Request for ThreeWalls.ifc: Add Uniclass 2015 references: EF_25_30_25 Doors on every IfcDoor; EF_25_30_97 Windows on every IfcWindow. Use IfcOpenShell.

First a look at what the model holds.

```python
import ifcopenshell

model = ifcopenshell.open("ThreeWalls.ifc")
print(model.schema)
print("classifications:", [c.Name for c in model.by_type("IfcClassification")])
for ifc_class in ("IfcDoor", "IfcRoof", "IfcStair", "IfcWall", "IfcWindow"):
    print(ifc_class, len(model.by_type(ifc_class)))
```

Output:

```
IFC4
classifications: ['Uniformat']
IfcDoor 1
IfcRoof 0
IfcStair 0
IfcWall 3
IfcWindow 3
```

```python
import ifcopenshell
import ifcopenshell.api.classification

model = ifcopenshell.open("ThreeWalls.ifc")

system = ifcopenshell.api.classification.add_classification(model, classification="Uniclass 2015")

codes = {
    "IfcDoor": ("EF_25_30_25", "Doors"),
    "IfcWindow": ("EF_25_30_97", "Windows"),
}
for ifc_class, (code, name) in codes.items():
    products = model.by_type(ifc_class)
    ifcopenshell.api.classification.add_reference(
        model, products=products, classification=system, identification=code, name=name
    )
    print(code, len(products))

model.write("ThreeWalls_rev.ifc")
```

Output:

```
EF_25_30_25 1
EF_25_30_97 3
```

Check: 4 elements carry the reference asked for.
